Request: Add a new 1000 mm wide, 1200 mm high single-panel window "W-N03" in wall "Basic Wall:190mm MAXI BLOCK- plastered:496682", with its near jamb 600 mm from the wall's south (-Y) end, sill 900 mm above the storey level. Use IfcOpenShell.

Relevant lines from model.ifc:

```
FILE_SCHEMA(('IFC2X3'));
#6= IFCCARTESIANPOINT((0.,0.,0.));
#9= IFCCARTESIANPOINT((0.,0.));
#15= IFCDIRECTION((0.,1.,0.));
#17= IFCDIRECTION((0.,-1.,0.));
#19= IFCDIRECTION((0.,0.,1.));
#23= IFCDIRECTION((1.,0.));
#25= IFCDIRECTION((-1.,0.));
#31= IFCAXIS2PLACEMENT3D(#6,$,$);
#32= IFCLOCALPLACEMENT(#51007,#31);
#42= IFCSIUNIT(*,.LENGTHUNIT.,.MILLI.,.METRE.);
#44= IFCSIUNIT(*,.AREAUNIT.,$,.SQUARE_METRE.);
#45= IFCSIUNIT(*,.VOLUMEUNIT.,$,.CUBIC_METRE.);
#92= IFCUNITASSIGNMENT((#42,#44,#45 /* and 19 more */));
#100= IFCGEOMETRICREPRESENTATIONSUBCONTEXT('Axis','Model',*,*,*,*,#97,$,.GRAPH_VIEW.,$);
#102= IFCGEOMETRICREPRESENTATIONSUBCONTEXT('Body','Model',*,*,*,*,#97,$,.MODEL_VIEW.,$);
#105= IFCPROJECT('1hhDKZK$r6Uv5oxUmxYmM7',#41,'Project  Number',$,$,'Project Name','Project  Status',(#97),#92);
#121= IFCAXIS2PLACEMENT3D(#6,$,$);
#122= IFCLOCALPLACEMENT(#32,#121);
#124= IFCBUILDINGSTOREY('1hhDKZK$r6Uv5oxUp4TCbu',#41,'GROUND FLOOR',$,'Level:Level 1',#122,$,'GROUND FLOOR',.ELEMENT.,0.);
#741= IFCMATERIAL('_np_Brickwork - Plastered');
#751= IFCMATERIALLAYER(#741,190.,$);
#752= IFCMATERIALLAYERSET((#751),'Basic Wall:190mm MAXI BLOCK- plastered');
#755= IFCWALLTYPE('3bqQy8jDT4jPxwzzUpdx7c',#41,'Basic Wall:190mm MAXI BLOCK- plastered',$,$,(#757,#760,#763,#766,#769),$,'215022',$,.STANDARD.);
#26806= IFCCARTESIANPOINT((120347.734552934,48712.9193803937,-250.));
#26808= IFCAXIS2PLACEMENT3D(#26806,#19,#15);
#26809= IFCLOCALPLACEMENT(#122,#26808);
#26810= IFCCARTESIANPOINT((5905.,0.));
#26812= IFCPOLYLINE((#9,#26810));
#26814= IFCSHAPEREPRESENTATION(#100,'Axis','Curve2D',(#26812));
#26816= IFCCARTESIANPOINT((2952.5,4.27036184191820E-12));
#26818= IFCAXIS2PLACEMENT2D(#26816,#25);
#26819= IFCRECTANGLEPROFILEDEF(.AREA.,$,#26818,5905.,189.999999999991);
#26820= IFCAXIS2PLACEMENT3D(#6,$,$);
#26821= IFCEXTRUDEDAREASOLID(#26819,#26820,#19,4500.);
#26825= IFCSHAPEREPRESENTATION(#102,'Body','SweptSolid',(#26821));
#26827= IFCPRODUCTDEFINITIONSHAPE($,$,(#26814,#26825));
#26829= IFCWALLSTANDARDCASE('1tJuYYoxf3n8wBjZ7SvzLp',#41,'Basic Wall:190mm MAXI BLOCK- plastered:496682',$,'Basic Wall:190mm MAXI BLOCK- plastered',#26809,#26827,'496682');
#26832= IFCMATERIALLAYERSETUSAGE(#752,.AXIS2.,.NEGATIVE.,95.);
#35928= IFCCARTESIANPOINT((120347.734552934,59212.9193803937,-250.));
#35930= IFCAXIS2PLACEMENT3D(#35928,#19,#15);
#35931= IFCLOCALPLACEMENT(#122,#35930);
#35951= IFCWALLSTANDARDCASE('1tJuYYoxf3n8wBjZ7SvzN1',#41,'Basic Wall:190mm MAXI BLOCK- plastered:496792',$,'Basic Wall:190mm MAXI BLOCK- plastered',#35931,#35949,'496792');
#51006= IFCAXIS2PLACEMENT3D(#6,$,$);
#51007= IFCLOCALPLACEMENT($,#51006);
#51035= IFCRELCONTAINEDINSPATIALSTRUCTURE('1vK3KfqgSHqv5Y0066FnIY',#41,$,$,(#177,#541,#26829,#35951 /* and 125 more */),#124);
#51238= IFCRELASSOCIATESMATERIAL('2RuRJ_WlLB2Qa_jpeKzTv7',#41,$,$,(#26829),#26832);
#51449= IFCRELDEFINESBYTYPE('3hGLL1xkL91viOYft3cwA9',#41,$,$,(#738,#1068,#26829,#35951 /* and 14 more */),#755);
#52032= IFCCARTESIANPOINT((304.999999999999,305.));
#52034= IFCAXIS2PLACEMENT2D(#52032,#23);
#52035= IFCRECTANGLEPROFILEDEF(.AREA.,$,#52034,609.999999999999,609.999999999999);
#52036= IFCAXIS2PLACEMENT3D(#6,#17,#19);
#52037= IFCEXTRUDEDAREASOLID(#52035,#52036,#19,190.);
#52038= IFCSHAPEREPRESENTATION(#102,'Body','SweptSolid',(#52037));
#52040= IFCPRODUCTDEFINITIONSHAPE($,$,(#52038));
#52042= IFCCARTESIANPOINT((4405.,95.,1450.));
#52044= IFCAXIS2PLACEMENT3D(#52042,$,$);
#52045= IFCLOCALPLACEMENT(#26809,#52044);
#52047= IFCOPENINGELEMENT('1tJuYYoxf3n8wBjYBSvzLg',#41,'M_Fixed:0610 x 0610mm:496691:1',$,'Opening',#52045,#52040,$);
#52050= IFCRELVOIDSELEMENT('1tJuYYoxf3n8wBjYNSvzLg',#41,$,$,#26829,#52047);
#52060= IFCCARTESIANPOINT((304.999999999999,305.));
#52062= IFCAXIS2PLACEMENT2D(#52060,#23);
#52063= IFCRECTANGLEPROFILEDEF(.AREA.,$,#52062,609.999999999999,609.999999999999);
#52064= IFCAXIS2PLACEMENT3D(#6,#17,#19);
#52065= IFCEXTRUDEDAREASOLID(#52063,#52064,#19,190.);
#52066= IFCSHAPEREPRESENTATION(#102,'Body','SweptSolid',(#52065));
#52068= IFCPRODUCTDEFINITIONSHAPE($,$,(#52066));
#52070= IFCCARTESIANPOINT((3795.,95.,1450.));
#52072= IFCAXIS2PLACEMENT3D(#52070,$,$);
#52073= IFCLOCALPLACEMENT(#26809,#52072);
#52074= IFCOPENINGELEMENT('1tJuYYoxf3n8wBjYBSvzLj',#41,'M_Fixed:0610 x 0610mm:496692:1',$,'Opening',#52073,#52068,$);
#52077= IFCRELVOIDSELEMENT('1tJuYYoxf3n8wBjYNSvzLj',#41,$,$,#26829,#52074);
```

```python
import numpy as np
import ifcopenshell
import ifcopenshell.api.feature
import ifcopenshell.api.geometry
import ifcopenshell.api.root
import ifcopenshell.api.spatial
import ifcopenshell.api.type
import ifcopenshell.geom
import ifcopenshell.util.element
import ifcopenshell.util.placement
import ifcopenshell.util.representation
import ifcopenshell.util.shape
import ifcopenshell.util.unit

model = ifcopenshell.open("model.ifc")
unit_scale = ifcopenshell.util.unit.calculate_unit_scale(model)
settings = ifcopenshell.geom.settings()


def volume(element):
    """Net volume in cubic metres, openings subtracted."""
    shape = ifcopenshell.geom.create_shape(settings, element)
    return ifcopenshell.util.shape.get_volume(shape.geometry)


wall = model.by_guid("1tJuYYoxf3n8wBjZ7SvzLp")
storey = ifcopenshell.util.element.get_container(wall, ifc_class="IfcBuildingStorey")
context = ifcopenshell.util.representation.get_context(model, "Model", "Body", "MODEL_VIEW")
before = volume(wall)

width, height, from_end, sill = 1, 1.2, 0.6, 0.9  # metres

# The wall runs along its own X axis, and the end named is its -X end.
wall_shape = ifcopenshell.geom.create_shape(settings, wall)
x, y, z = ifcopenshell.util.shape.get_vertices(wall_shape.geometry).T
start = x.min() + from_end
face, thickness = float(y.min()), float(y.max() - y.min())
wall_matrix = ifcopenshell.util.placement.get_local_placement(wall.ObjectPlacement)
level = ifcopenshell.util.placement.get_local_placement(storey.ObjectPlacement)[2, 3]


def in_wall(x, y):
    """Placement at x, y metres in the wall's axes, at sill height."""
    matrix = wall_matrix.copy()
    matrix[:, 3] = wall_matrix @ np.array([x / unit_scale, y / unit_scale, 0.0, 1.0])
    matrix[2, 3] = level + sill / unit_scale
    return matrix


# Opening: a box that overshoots both wall faces by 50 mm.
opening = ifcopenshell.api.root.create_entity(model, ifc_class="IfcOpeningElement")
box = ifcopenshell.api.geometry.add_wall_representation(
    model, context=context, length=width, height=height, thickness=thickness + 0.1
)
ifcopenshell.api.geometry.assign_representation(model, product=opening, representation=box)
ifcopenshell.api.geometry.edit_object_placement(model, product=opening, matrix=in_wall(start, face - 0.05), is_si=False)
ifcopenshell.api.feature.add_feature(model, feature=opening, element=wall)

window = ifcopenshell.api.root.create_entity(model, ifc_class="IfcWindow", name="W-N03")
window.OverallWidth, window.OverallHeight = width / unit_scale, height / unit_scale
body = ifcopenshell.api.geometry.add_window_representation(
    model,
    context=context,
    overall_width=window.OverallWidth,
    overall_height=window.OverallHeight,
    partition_type="SINGLE_PANEL",
)
ifcopenshell.api.geometry.assign_representation(model, product=window, representation=body)
ifcopenshell.api.spatial.assign_container(model, products=[window], relating_structure=storey)
fills = ifcopenshell.api.feature.add_filling(model, opening=opening, element=window)
fills.OwnerHistory = window.OwnerHistory  # required in IFC2X3

# IFC2X3 keeps the operation on the window style.
style = ifcopenshell.api.root.create_entity(model, ifc_class="IfcWindowStyle", name="W-N03")
style.OperationType, style.ConstructionType = "SINGLE_PANEL", "NOTDEFINED"
style.ParameterTakesPrecedence = style.Sizeable = False
ifcopenshell.api.type.assign_type(model, related_objects=[window], relating_type=style)

# Centre the window in the wall's thickness.
ifcopenshell.api.geometry.edit_object_placement(model, product=window, matrix=in_wall(start, face), is_si=False)
window_shape = ifcopenshell.geom.create_shape(settings, window)
depth = ifcopenshell.util.shape.get_vertices(window_shape.geometry)[:, 1]
offset = face + thickness / 2 - (depth.min() + depth.max()) / 2
ifcopenshell.api.geometry.edit_object_placement(model, product=window, matrix=in_wall(start, offset), is_si=False)

after = volume(wall)

print(f"wall volume {before:.3f} -> {after:.3f} m3")

model.write("model_updated.ifc")
```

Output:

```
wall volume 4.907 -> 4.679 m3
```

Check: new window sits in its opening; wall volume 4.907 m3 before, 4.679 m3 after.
